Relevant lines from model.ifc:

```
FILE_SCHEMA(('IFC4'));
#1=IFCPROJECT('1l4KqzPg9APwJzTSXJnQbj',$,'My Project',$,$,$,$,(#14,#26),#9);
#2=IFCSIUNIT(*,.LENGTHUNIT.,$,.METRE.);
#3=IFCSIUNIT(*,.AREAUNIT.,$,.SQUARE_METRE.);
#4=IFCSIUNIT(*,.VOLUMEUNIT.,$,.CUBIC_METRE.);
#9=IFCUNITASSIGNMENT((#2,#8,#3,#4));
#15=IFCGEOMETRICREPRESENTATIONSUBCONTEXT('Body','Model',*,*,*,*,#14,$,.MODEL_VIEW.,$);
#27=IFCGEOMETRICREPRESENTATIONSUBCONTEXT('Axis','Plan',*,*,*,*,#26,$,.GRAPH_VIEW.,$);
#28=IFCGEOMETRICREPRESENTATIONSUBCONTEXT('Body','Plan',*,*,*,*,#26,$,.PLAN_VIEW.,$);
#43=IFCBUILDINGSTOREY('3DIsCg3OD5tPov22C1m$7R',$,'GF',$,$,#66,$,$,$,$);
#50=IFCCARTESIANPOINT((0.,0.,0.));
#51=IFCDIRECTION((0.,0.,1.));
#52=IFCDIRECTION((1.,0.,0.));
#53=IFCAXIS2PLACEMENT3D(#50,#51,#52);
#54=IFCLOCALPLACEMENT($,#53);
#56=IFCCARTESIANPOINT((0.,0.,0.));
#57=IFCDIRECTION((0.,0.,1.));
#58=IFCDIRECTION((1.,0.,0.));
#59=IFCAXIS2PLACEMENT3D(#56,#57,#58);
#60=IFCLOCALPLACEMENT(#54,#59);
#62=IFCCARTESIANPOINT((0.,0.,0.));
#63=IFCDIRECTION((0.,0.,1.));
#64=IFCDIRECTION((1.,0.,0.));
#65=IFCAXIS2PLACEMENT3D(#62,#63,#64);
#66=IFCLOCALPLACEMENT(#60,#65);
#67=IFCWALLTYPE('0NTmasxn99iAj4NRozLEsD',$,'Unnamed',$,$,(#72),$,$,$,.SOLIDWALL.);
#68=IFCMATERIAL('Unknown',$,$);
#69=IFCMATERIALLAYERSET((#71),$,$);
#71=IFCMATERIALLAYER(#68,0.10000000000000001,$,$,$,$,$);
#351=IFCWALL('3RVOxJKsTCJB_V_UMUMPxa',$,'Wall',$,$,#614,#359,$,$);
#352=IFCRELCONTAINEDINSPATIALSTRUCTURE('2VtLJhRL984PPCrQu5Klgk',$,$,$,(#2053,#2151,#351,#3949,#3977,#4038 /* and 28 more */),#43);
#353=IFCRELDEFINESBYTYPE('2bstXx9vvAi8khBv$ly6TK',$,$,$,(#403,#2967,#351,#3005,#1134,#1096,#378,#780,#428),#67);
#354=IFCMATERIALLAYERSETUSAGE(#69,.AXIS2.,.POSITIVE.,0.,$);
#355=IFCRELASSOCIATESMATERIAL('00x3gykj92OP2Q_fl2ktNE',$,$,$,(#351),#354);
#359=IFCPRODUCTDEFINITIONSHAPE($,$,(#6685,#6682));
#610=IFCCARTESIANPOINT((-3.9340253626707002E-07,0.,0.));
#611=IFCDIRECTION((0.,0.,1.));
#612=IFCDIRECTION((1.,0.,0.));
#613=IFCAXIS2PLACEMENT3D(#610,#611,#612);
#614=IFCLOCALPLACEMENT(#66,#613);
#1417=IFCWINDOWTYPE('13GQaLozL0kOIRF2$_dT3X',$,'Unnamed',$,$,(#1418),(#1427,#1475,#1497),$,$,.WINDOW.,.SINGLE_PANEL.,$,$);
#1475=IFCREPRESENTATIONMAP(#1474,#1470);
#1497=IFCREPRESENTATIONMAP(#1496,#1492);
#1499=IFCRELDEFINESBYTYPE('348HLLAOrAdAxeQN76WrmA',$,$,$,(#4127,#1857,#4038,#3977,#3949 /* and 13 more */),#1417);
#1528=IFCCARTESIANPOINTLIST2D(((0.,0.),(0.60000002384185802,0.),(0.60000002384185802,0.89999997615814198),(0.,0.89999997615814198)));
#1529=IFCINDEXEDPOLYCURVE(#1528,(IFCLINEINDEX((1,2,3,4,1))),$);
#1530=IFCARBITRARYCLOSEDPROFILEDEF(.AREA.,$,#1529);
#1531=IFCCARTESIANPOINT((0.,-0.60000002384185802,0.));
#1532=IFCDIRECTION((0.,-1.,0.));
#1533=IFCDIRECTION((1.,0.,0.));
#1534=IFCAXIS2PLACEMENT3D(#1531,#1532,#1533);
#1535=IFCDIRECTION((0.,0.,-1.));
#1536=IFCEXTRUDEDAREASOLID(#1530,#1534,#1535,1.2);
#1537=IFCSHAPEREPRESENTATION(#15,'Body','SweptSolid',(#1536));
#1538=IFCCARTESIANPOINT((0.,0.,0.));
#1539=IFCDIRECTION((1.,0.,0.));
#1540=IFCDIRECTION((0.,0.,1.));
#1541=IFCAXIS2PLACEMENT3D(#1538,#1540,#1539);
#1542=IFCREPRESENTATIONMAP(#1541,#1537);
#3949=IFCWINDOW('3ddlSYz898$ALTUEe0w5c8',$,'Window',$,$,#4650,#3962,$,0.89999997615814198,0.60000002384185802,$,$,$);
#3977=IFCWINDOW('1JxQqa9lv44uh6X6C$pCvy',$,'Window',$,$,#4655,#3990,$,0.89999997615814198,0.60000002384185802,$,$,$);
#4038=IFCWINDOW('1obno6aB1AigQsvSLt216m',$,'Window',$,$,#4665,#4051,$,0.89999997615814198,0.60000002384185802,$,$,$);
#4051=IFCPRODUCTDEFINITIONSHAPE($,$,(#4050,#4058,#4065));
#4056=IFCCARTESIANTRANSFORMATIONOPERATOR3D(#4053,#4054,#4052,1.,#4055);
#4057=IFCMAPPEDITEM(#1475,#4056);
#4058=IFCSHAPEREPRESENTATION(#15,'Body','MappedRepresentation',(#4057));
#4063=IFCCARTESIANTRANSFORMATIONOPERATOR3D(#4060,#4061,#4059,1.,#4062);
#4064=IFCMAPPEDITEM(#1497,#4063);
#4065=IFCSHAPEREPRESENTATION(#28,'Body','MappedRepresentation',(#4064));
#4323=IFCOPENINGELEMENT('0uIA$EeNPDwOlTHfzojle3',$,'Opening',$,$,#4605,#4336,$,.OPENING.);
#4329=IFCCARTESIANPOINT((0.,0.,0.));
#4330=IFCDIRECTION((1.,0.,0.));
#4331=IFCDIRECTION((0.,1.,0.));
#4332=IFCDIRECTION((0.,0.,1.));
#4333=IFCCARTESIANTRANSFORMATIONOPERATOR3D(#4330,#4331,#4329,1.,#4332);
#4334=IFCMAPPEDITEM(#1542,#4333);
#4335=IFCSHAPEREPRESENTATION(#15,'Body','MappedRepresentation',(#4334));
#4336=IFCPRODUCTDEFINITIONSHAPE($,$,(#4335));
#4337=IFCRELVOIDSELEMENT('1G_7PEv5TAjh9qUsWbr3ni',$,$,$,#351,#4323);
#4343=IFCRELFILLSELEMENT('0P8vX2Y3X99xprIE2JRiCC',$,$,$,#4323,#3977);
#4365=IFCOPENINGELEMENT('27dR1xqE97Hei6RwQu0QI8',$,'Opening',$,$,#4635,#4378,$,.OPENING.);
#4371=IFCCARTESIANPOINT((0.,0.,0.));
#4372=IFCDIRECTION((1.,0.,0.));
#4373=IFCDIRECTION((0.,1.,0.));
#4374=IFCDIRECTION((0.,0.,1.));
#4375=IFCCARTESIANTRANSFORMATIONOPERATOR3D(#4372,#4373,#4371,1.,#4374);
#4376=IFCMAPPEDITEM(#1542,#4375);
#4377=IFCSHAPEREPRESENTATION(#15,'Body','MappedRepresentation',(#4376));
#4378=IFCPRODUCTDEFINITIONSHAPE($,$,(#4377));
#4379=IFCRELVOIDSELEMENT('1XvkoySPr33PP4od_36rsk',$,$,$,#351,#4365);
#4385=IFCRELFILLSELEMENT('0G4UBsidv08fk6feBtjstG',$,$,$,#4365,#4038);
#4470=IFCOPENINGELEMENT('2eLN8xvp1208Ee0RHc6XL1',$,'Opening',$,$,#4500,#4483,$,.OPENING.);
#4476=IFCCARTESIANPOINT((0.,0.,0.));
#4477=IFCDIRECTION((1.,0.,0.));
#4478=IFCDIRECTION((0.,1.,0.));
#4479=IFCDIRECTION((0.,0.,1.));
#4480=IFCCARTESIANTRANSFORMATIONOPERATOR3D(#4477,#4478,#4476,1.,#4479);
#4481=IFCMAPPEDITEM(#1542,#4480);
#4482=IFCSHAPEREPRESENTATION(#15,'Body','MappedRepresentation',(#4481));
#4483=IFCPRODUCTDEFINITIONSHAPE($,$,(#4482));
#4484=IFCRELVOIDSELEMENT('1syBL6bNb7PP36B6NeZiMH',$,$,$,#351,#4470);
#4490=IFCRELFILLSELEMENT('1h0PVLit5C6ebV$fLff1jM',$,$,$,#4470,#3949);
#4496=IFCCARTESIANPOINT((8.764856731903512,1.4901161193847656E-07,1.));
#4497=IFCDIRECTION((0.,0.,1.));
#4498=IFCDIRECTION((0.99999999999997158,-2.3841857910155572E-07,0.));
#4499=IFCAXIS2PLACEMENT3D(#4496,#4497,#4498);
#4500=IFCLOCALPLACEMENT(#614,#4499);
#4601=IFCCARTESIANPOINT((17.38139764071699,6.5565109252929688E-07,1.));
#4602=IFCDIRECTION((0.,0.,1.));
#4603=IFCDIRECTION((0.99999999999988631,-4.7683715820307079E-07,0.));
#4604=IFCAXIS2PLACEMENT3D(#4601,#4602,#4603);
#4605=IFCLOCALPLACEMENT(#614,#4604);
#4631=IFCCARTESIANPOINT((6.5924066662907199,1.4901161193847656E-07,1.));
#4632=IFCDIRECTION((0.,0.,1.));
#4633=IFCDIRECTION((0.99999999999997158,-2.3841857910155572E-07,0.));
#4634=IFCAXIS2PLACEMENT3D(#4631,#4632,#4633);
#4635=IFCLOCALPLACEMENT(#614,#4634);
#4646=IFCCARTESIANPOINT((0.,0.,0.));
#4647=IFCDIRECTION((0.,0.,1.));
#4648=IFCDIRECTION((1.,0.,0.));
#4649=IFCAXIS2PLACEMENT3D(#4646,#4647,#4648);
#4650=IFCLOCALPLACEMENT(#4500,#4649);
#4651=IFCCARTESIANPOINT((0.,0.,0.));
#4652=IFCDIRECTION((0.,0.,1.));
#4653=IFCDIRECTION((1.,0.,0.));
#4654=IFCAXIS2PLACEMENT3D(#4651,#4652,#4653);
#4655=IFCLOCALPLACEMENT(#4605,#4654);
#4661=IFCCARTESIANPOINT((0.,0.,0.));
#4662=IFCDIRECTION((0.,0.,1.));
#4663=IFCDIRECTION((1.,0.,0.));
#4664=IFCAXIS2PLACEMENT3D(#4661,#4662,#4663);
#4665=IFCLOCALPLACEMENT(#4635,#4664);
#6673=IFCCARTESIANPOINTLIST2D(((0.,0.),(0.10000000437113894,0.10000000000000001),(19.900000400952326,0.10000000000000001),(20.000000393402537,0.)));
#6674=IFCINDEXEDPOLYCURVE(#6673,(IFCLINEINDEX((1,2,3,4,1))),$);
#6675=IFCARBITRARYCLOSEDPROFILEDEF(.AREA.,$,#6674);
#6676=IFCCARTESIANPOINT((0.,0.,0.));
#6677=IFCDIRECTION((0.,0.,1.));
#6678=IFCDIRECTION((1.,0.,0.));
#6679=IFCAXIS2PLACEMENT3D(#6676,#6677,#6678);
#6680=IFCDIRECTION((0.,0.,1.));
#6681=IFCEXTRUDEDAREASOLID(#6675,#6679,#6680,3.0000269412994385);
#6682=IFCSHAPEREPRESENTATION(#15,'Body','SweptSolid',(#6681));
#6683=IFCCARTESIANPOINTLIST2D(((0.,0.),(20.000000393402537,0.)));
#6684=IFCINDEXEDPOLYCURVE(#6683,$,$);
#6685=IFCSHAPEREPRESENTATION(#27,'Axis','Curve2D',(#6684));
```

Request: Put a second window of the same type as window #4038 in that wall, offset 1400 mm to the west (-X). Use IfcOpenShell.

```python
import ifcopenshell
import ifcopenshell.api.feature
import ifcopenshell.api.geometry
import ifcopenshell.api.root
import ifcopenshell.geom
import ifcopenshell.util.element
import ifcopenshell.util.placement
import ifcopenshell.util.shape

model = ifcopenshell.open("model.ifc")
settings = ifcopenshell.geom.settings()


def volume(element):
    """Net volume in cubic metres, openings subtracted."""
    shape = ifcopenshell.geom.create_shape(settings, element)
    return ifcopenshell.util.shape.get_volume(shape.geometry)


window = model.by_guid("1obno6aB1AigQsvSLt216m")
opening = window.FillsVoids[0].RelatingOpeningElement
wall = opening.VoidsElements[0].RelatingBuildingElement
before = volume(wall)
shift = ifcopenshell.util.placement.get_local_placement(wall.ObjectPlacement)[:3, 0] * -1.4

# copy_class copies the void relationship, type, container and properties, but no geometry.
new_opening = ifcopenshell.api.root.copy_class(model, product=opening)
new_opening.Representation = ifcopenshell.util.element.copy_deep(
    model, opening.Representation, exclude=["IfcGeometricRepresentationContext", "IfcRepresentationMap"]
)
new_window = ifcopenshell.api.root.copy_class(model, product=window)
new_window.Representation = ifcopenshell.util.element.copy_deep(
    model, window.Representation, exclude=["IfcGeometricRepresentationContext", "IfcRepresentationMap"]
)
ifcopenshell.api.feature.add_filling(model, opening=new_opening, element=new_window)

for old, new in ((opening, new_opening), (window, new_window)):
    matrix = ifcopenshell.util.placement.get_local_placement(old.ObjectPlacement)
    matrix[:3, 3] += shift
    ifcopenshell.api.geometry.edit_object_placement(model, product=new, matrix=matrix, is_si=False)

after = volume(wall)

print(f"wall volume {before:.3f} -> {after:.3f} m3")

model.write("model_edited.ifc")
```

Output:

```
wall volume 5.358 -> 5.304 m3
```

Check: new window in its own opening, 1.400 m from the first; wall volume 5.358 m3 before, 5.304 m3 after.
